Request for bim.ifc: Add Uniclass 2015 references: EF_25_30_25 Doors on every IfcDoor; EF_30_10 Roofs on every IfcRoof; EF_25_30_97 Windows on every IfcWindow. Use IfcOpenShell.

First a look at what the model holds.

```python
import ifcopenshell

model = ifcopenshell.open("bim.ifc")
print(model.schema)
print("classifications:", [c.Name for c in model.by_type("IfcClassification")])
for ifc_class in ("IfcDoor", "IfcRoof", "IfcStair", "IfcWall", "IfcWindow"):
    print(ifc_class, len(model.by_type(ifc_class)))
```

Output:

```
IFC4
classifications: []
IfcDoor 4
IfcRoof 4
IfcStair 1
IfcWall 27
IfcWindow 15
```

```python
import ifcopenshell
import ifcopenshell.api.classification

model = ifcopenshell.open("bim.ifc")

system = ifcopenshell.api.classification.add_classification(model, classification="Uniclass 2015")

codes = {
    "IfcDoor": ("EF_25_30_25", "Doors"),
    "IfcRoof": ("EF_30_10", "Roofs"),
    "IfcWindow": ("EF_25_30_97", "Windows"),
}
for ifc_class, (code, name) in codes.items():
    products = model.by_type(ifc_class)
    ifcopenshell.api.classification.add_reference(
        model, products=products, classification=system, identification=code, name=name
    )
    print(code, len(products))

model.write("bim_updated.ifc")
```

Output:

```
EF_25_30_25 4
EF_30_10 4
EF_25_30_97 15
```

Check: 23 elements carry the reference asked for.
